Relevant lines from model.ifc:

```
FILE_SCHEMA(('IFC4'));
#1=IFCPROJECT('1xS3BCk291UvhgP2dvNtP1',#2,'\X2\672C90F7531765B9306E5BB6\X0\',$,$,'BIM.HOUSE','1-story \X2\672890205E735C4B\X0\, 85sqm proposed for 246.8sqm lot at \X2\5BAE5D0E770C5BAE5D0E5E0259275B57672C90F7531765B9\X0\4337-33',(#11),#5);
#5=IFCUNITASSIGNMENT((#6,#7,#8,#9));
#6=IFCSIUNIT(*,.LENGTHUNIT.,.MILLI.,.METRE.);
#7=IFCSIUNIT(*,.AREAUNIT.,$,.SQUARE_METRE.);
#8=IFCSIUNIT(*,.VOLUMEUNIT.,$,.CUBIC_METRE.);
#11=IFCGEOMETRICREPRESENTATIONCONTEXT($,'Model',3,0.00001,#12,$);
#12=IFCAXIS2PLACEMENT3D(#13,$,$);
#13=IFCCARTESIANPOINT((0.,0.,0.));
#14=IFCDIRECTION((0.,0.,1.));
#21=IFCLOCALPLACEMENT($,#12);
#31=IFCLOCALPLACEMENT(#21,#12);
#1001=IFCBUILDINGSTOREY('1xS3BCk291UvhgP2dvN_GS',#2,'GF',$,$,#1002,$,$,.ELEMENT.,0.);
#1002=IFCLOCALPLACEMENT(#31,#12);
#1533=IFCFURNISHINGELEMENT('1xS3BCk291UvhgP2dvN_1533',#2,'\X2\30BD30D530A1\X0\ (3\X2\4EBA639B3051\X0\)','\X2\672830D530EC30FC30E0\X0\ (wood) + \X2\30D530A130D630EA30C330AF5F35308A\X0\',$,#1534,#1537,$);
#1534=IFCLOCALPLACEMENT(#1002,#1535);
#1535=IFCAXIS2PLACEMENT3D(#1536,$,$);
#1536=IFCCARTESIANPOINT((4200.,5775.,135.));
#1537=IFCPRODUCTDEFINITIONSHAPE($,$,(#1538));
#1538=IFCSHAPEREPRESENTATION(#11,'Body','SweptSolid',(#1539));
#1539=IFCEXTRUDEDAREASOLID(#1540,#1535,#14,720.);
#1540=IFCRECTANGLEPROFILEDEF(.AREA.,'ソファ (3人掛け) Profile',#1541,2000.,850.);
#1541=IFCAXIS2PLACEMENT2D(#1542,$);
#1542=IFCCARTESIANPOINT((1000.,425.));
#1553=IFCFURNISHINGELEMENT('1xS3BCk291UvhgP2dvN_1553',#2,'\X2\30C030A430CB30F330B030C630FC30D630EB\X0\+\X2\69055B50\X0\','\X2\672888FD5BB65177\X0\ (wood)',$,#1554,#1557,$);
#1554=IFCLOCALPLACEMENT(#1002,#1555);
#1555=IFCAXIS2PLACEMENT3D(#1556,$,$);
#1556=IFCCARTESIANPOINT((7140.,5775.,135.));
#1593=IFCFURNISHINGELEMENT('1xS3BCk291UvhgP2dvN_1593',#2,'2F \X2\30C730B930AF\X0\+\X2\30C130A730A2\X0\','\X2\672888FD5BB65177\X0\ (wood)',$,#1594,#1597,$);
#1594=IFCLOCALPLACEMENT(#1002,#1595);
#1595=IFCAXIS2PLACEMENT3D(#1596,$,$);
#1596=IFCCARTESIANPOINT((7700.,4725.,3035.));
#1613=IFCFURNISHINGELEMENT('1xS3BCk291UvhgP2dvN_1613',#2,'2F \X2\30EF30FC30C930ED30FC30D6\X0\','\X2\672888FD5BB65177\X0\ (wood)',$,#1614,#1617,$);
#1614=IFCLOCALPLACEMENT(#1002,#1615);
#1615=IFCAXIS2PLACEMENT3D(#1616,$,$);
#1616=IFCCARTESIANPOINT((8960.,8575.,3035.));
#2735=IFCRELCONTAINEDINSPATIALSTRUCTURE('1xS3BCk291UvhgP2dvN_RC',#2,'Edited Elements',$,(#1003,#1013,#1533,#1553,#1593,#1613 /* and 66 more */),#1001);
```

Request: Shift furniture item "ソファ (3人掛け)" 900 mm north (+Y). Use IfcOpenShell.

```python
import ifcopenshell
import ifcopenshell.api.geometry
import ifcopenshell.util.placement

model = ifcopenshell.open("model.ifc")

item = model.by_guid("1xS3BCk291UvhgP2dvN_1533")
matrix = ifcopenshell.util.placement.get_local_placement(item.ObjectPlacement)
matrix[1, 3] += 900.0
ifcopenshell.api.geometry.edit_object_placement(model, product=item, matrix=matrix, is_si=False)

print(ifcopenshell.util.placement.get_local_placement(item.ObjectPlacement).round(3) + 0.0)

model.write("model-out.ifc")
```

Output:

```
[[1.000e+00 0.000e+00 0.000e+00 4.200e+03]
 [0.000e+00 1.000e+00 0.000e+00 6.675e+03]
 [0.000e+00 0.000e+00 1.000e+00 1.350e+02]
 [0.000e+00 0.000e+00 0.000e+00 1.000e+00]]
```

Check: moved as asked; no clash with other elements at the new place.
